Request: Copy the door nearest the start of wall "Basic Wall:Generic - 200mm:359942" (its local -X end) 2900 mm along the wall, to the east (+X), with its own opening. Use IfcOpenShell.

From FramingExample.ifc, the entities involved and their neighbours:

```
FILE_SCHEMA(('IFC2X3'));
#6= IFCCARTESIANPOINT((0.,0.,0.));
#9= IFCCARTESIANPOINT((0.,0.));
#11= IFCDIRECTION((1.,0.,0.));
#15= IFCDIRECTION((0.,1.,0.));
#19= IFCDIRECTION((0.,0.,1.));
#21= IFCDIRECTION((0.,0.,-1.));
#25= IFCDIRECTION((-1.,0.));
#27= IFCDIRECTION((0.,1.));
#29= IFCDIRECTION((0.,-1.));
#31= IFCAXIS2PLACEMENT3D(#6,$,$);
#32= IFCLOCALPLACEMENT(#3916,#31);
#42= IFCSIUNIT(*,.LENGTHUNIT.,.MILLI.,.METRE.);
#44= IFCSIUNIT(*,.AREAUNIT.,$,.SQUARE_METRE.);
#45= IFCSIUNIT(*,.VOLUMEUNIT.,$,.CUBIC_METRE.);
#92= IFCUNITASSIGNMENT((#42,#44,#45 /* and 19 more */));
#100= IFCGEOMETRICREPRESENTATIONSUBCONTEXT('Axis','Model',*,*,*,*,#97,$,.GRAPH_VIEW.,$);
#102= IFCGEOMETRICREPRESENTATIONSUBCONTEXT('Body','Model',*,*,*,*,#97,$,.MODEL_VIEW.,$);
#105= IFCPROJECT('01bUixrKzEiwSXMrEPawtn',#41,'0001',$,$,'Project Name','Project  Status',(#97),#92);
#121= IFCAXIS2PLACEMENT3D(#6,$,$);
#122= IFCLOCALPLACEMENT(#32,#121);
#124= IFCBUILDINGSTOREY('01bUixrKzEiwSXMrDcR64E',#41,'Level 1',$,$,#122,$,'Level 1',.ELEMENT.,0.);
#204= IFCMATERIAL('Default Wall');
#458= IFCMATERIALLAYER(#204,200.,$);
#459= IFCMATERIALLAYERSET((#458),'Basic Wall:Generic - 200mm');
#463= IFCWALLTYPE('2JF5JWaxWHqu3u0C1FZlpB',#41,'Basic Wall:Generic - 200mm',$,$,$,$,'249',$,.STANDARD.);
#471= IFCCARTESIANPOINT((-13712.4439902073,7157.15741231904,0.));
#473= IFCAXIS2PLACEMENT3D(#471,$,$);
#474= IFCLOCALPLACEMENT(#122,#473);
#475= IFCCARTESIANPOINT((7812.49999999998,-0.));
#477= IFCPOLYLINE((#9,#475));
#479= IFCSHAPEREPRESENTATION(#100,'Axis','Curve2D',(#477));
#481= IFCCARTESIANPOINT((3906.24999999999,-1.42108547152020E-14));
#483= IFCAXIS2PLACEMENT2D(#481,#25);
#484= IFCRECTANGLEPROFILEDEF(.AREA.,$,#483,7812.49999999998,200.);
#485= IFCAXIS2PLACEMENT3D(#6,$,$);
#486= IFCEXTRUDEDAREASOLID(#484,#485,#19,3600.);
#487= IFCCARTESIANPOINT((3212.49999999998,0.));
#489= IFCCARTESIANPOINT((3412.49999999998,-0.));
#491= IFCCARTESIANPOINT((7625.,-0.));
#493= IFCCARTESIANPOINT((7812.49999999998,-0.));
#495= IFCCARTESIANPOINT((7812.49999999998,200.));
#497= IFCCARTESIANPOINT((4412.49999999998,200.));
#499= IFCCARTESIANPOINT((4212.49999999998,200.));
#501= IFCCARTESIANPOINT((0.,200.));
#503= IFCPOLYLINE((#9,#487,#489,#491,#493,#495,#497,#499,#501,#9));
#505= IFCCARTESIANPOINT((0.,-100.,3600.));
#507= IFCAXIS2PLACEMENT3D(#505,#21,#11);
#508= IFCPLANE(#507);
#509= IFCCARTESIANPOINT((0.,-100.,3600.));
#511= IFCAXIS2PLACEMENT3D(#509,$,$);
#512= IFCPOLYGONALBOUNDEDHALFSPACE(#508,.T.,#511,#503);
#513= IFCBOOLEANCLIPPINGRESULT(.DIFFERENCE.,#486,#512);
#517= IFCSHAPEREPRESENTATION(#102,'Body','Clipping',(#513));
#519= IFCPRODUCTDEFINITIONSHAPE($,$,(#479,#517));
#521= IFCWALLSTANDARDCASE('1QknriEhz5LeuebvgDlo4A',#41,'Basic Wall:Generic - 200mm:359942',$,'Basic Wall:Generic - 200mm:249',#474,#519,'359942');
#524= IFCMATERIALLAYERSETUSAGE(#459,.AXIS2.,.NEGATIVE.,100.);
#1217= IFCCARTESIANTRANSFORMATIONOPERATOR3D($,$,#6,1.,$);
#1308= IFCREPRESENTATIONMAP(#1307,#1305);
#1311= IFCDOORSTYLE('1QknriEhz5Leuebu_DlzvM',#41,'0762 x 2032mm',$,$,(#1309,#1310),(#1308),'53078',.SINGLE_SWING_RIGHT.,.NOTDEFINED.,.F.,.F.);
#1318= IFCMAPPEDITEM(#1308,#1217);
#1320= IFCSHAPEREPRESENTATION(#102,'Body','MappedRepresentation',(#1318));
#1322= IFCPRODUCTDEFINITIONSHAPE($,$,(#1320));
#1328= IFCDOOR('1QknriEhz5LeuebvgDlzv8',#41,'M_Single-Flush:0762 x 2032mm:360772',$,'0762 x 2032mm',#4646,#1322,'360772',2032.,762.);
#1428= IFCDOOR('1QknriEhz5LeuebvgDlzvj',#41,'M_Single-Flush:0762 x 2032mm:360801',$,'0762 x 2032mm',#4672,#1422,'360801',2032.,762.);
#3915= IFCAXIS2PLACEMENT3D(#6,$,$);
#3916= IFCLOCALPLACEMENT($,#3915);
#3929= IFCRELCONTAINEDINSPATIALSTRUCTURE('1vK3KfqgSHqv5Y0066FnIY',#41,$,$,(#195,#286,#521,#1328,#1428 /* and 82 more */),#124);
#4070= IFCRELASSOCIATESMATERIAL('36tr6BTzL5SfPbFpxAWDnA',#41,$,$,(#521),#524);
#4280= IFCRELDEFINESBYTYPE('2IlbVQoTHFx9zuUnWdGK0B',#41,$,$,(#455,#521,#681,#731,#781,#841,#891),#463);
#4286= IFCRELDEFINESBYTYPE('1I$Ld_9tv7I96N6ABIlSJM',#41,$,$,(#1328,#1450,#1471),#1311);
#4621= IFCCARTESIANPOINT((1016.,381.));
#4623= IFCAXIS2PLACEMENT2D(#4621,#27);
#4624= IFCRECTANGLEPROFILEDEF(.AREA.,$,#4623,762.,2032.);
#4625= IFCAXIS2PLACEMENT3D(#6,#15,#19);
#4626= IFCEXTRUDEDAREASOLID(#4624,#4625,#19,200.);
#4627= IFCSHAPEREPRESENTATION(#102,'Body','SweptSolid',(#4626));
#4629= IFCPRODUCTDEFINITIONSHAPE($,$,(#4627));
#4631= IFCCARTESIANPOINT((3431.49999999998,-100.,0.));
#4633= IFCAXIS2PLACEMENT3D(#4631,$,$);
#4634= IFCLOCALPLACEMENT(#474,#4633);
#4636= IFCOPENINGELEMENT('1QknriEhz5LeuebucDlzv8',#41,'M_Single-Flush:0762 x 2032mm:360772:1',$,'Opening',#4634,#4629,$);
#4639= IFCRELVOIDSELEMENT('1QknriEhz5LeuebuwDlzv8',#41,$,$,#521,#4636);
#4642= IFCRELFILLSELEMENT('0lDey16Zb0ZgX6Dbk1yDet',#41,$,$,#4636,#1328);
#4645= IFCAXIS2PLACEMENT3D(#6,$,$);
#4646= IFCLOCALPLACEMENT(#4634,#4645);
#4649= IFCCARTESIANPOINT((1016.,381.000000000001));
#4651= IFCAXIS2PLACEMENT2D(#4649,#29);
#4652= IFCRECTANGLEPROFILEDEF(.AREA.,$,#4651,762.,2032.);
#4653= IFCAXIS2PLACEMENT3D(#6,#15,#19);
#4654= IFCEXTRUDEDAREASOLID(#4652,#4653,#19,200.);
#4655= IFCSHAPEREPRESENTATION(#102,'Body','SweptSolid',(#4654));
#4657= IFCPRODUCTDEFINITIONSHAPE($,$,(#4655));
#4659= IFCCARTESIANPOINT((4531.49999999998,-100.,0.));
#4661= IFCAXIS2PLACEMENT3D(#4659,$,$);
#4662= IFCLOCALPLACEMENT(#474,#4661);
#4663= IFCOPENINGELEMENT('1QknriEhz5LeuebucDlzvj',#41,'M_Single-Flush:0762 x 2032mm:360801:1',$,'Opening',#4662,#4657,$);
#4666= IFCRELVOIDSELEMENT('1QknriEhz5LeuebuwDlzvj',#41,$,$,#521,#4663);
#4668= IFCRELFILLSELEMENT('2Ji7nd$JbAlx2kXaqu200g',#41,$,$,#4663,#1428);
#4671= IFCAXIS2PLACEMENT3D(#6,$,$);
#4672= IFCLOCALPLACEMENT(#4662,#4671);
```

```python
import ifcopenshell
import ifcopenshell.api.feature
import ifcopenshell.api.geometry
import ifcopenshell.api.root
import ifcopenshell.geom
import ifcopenshell.util.element
import ifcopenshell.util.placement
import ifcopenshell.util.shape
import ifcopenshell.util.unit

model = ifcopenshell.open("FramingExample.ifc")
unit_scale = ifcopenshell.util.unit.calculate_unit_scale(model)
settings = ifcopenshell.geom.settings()


def volume(element):
    """Net volume in cubic metres, openings subtracted."""
    shape = ifcopenshell.geom.create_shape(settings, element)
    return ifcopenshell.util.shape.get_volume(shape.geometry)


def reuse_history(source, copy):
    """copy_class also copies each property set's owner history, people and application; keep the originals."""
    for rel in copy.IsDefinedBy:
        if rel.is_a("IfcRelDefinesByProperties") and (history := rel.RelatingPropertyDefinition.OwnerHistory):
            rel.RelatingPropertyDefinition.OwnerHistory = source.OwnerHistory
            ifcopenshell.util.element.remove_deep2(model, history)


door = model.by_guid("1QknriEhz5LeuebvgDlzv8")
opening = door.FillsVoids[0].RelatingOpeningElement
wall = opening.VoidsElements[0].RelatingBuildingElement
before = volume(wall)
shift = ifcopenshell.util.placement.get_local_placement(wall.ObjectPlacement)[:3, 0] * 2.9 / unit_scale

# copy_class copies the void relationship, type, container and properties, but no geometry.
new_opening = ifcopenshell.api.root.copy_class(model, product=opening)
new_opening.Representation = ifcopenshell.util.element.copy_deep(
    model, opening.Representation, exclude=["IfcGeometricRepresentationContext", "IfcRepresentationMap"]
)
new_opening.Name = "M_Single-Flush:0762 x 2032mm"
new_door = ifcopenshell.api.root.copy_class(model, product=door)
new_door.Representation = ifcopenshell.util.element.copy_deep(
    model, door.Representation, exclude=["IfcGeometricRepresentationContext", "IfcRepresentationMap"]
)
new_door.Name = "M_Single-Flush:0762 x 2032mm"
new_door.Tag = None
reuse_history(door, new_door)
fills = ifcopenshell.api.feature.add_filling(model, opening=new_opening, element=new_door)
fills.OwnerHistory = new_door.OwnerHistory  # required in IFC2X3

for old, new in ((opening, new_opening), (door, new_door)):
    matrix = ifcopenshell.util.placement.get_local_placement(old.ObjectPlacement)
    matrix[:3, 3] += shift
    ifcopenshell.api.geometry.edit_object_placement(model, product=new, matrix=matrix, is_si=False)

after = volume(wall)

print(f"wall volume {before:.3f} -> {after:.3f} m3")

model.write("FramingExample_edited.ifc")
```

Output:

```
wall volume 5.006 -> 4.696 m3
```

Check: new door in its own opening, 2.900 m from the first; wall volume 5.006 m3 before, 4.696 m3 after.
